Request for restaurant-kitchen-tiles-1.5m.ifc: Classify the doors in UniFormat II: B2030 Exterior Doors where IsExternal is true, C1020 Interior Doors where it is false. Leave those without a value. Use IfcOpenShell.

First a look at what the model holds.

```python
import ifcopenshell
import ifcopenshell.util.element

model = ifcopenshell.open("restaurant-kitchen-tiles-1.5m.ifc")
print(model.schema)
print("classifications:", [c.Name for c in model.by_type("IfcClassification")])
values = [ifcopenshell.util.element.get_pset(e, "Pset_DoorCommon", "IsExternal") for e in model.by_type("IfcDoor")]
for value in (True, False, None):
    print("IsExternal", value, values.count(value))
```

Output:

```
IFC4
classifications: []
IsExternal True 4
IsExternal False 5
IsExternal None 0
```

```python
import ifcopenshell
import ifcopenshell.api.classification
import ifcopenshell.util.element

model = ifcopenshell.open("restaurant-kitchen-tiles-1.5m.ifc")

system = ifcopenshell.api.classification.add_classification(model, classification="UniFormat II")

doors = model.by_type("IfcDoor")
external = {e: ifcopenshell.util.element.get_pset(e, "Pset_DoorCommon", "IsExternal") for e in doors}
for flag, code, name in ((True, "B2030", "Exterior Doors"), (False, "C1020", "Interior Doors")):
    products = [e for e in doors if external[e] is flag]
    ifcopenshell.api.classification.add_reference(
        model, products=products, classification=system, identification=code, name=name
    )
    print(code, len(products))

model.write("restaurant-kitchen-tiles-1.5m_updated.ifc")
```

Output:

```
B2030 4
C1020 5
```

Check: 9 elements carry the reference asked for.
